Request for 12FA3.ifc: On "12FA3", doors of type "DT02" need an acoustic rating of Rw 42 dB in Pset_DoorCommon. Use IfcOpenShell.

First a look at what the model holds.

```python
import ifcopenshell
import ifcopenshell.util.element

model = ifcopenshell.open("12FA3.ifc")
print(model.schema)
storey = next(s for s in model.by_type("IfcBuildingStorey") if s.Name == "12FA3")
doors = [e for e in ifcopenshell.util.element.get_decomposition(storey) if e.is_a("IfcDoor")]
seen = {}
for e in doors:
    element_type = ifcopenshell.util.element.get_type(e)
    key = (element_type.Name if element_type != e and element_type else None, ifcopenshell.util.element.get_pset(e, "Pset_DoorCommon", "AcousticRating"))
    seen[key] = seen.get(key, 0) + 1
for (name, value), count in sorted(seen.items(), key=str):
    print(count, "x", name, "|", value)
```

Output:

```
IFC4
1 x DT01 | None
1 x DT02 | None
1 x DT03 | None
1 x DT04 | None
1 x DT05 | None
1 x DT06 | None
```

```python
import ifcopenshell
import ifcopenshell.api.pset
import ifcopenshell.util.element

model = ifcopenshell.open("12FA3.ifc")

storey = next(s for s in model.by_type("IfcBuildingStorey") if s.Name == "12FA3")
doors = [e for e in ifcopenshell.util.element.get_decomposition(storey) if e.is_a("IfcDoor")]

count = 0
for e in doors:
    element_type = ifcopenshell.util.element.get_type(e)
    if element_type in (None, e) or element_type.Name != "DT02":
        continue
    # add_pset returns the element's existing set when there is one.
    pset = ifcopenshell.api.pset.add_pset(model, product=e, name="Pset_DoorCommon")
    ifcopenshell.api.pset.edit_pset(model, pset=pset, properties={"AcousticRating": "Rw 42 dB"})
    count += 1

print(count, "doors updated")

model.write("12FA3_rev.ifc")
```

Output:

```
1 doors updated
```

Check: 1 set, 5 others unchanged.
